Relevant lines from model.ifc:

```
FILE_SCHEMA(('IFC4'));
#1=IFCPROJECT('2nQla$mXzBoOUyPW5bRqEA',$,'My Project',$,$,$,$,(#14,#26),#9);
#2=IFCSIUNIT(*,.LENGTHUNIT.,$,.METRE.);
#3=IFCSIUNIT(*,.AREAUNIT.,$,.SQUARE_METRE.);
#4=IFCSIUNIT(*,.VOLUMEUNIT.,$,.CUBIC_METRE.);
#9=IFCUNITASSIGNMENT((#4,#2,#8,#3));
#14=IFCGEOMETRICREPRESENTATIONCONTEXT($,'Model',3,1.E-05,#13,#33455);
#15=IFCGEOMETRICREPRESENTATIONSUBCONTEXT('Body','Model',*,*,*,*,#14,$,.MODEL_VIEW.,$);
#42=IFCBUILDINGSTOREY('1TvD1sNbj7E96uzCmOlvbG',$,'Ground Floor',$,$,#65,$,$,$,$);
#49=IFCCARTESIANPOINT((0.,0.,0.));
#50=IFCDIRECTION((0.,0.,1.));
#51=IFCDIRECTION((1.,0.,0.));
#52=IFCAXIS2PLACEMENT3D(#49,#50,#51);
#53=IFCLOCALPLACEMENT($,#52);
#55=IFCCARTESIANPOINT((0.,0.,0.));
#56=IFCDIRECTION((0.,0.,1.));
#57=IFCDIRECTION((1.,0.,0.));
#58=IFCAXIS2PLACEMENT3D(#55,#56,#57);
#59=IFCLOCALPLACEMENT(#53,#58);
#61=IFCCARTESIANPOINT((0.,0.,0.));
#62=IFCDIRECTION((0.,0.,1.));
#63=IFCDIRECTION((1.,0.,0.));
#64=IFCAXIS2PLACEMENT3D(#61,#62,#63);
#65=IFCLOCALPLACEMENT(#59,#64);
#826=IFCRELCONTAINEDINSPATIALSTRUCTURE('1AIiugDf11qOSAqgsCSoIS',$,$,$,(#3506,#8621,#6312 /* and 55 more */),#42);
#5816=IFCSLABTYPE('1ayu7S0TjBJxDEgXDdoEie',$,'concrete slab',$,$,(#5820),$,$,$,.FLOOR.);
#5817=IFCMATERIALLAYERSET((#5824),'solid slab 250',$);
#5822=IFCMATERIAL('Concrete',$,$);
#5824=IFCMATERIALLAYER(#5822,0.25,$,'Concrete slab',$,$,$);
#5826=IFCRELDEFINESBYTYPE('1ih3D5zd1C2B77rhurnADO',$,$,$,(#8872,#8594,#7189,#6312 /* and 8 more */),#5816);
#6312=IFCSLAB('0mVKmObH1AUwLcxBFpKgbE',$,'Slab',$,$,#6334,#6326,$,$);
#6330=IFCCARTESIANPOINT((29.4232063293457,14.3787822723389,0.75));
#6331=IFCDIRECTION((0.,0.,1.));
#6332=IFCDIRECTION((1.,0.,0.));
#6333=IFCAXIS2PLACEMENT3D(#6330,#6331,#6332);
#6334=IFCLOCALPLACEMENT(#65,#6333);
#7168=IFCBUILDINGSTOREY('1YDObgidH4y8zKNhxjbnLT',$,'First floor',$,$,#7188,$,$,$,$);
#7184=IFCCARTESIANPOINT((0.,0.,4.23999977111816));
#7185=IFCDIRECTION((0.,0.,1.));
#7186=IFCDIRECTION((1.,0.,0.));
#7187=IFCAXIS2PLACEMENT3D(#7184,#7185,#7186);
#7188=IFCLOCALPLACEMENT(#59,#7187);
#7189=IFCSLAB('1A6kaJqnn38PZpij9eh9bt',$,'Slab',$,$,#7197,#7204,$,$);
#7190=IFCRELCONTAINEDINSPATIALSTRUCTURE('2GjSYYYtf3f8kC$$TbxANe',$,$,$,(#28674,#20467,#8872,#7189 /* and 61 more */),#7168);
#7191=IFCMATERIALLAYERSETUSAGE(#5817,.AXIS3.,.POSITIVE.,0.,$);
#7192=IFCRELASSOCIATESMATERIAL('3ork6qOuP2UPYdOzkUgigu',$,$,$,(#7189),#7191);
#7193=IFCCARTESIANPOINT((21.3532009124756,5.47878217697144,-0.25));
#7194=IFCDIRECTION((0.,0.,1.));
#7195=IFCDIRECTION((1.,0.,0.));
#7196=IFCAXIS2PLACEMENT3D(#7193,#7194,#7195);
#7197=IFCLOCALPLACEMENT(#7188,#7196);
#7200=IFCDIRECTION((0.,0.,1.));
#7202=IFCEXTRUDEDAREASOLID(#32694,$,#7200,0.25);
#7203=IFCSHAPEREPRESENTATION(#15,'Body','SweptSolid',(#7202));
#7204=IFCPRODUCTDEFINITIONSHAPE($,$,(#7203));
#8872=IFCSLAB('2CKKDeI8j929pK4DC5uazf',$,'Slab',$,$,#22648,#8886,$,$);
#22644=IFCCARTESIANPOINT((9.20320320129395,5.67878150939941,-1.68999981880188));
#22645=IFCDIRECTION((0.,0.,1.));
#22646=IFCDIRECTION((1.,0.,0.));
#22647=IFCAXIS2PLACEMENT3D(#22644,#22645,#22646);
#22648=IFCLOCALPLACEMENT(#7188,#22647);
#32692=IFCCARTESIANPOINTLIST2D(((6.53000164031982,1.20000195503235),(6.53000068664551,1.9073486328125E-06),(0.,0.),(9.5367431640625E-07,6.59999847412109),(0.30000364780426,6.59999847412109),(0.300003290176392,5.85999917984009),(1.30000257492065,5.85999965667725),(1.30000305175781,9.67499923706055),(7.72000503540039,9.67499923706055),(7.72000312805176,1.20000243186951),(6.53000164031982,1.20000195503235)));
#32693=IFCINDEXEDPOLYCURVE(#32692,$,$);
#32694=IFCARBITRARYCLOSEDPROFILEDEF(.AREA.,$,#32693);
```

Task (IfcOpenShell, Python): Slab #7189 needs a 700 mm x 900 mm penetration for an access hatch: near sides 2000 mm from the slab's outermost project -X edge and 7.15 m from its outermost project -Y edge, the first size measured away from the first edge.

```python
import numpy as np
import ifcopenshell
import ifcopenshell.api.feature
import ifcopenshell.api.geometry
import ifcopenshell.api.root
import ifcopenshell.geom
import ifcopenshell.util.placement
import ifcopenshell.util.representation
import ifcopenshell.util.shape
import ifcopenshell.util.unit

model = ifcopenshell.open("model.ifc")
unit_scale = ifcopenshell.util.unit.calculate_unit_scale(model)
settings = ifcopenshell.geom.settings()


def volume(element):
    """Net volume in cubic metres, openings subtracted."""
    shape = ifcopenshell.geom.create_shape(settings, element)
    return ifcopenshell.util.shape.get_volume(shape.geometry)


slab = model.by_id(7189)
before = volume(slab)

# Extent in the slab's own axes, in metres. The edges named are its -X and -Y sides.
slab_shape = ifcopenshell.geom.create_shape(settings, slab)
vertices = ifcopenshell.util.shape.get_vertices(slab_shape.geometry)
x_min, y_min, bottom = vertices.min(axis=0)
top = vertices[:, 2].max()

opening = ifcopenshell.api.root.create_entity(model, ifc_class="IfcOpeningElement", name="Access hatch opening", predefined_type="OPENING")
context = ifcopenshell.util.representation.get_context(model, "Model", "Body", "MODEL_VIEW")
width, depth = 0.7, 0.9
outline = [(0.0, 0.0), (width, 0.0), (width, depth), (0.0, depth), (0.0, 0.0)]
# Overshoot both faces by 50 mm so the cut is clean.
shape = ifcopenshell.api.geometry.add_slab_representation(
    model, context=context, depth=top - bottom + 0.1, polyline=outline
)
ifcopenshell.api.geometry.assign_representation(model, product=opening, representation=shape)

matrix = ifcopenshell.util.placement.get_local_placement(slab.ObjectPlacement)
matrix[:, 3] = matrix @ np.append(np.array([x_min + 2, y_min + 7.15, bottom - 0.05]) / unit_scale, 1.0)
ifcopenshell.api.geometry.edit_object_placement(model, product=opening, matrix=matrix, is_si=False)
ifcopenshell.api.feature.add_feature(model, feature=opening, element=slab)

after = volume(slab)

print(f"slab volume {before:.3f} -> {after:.3f} m3")

model.write("model_updated.ifc")
```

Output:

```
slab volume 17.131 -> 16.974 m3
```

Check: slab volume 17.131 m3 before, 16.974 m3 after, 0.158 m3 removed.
